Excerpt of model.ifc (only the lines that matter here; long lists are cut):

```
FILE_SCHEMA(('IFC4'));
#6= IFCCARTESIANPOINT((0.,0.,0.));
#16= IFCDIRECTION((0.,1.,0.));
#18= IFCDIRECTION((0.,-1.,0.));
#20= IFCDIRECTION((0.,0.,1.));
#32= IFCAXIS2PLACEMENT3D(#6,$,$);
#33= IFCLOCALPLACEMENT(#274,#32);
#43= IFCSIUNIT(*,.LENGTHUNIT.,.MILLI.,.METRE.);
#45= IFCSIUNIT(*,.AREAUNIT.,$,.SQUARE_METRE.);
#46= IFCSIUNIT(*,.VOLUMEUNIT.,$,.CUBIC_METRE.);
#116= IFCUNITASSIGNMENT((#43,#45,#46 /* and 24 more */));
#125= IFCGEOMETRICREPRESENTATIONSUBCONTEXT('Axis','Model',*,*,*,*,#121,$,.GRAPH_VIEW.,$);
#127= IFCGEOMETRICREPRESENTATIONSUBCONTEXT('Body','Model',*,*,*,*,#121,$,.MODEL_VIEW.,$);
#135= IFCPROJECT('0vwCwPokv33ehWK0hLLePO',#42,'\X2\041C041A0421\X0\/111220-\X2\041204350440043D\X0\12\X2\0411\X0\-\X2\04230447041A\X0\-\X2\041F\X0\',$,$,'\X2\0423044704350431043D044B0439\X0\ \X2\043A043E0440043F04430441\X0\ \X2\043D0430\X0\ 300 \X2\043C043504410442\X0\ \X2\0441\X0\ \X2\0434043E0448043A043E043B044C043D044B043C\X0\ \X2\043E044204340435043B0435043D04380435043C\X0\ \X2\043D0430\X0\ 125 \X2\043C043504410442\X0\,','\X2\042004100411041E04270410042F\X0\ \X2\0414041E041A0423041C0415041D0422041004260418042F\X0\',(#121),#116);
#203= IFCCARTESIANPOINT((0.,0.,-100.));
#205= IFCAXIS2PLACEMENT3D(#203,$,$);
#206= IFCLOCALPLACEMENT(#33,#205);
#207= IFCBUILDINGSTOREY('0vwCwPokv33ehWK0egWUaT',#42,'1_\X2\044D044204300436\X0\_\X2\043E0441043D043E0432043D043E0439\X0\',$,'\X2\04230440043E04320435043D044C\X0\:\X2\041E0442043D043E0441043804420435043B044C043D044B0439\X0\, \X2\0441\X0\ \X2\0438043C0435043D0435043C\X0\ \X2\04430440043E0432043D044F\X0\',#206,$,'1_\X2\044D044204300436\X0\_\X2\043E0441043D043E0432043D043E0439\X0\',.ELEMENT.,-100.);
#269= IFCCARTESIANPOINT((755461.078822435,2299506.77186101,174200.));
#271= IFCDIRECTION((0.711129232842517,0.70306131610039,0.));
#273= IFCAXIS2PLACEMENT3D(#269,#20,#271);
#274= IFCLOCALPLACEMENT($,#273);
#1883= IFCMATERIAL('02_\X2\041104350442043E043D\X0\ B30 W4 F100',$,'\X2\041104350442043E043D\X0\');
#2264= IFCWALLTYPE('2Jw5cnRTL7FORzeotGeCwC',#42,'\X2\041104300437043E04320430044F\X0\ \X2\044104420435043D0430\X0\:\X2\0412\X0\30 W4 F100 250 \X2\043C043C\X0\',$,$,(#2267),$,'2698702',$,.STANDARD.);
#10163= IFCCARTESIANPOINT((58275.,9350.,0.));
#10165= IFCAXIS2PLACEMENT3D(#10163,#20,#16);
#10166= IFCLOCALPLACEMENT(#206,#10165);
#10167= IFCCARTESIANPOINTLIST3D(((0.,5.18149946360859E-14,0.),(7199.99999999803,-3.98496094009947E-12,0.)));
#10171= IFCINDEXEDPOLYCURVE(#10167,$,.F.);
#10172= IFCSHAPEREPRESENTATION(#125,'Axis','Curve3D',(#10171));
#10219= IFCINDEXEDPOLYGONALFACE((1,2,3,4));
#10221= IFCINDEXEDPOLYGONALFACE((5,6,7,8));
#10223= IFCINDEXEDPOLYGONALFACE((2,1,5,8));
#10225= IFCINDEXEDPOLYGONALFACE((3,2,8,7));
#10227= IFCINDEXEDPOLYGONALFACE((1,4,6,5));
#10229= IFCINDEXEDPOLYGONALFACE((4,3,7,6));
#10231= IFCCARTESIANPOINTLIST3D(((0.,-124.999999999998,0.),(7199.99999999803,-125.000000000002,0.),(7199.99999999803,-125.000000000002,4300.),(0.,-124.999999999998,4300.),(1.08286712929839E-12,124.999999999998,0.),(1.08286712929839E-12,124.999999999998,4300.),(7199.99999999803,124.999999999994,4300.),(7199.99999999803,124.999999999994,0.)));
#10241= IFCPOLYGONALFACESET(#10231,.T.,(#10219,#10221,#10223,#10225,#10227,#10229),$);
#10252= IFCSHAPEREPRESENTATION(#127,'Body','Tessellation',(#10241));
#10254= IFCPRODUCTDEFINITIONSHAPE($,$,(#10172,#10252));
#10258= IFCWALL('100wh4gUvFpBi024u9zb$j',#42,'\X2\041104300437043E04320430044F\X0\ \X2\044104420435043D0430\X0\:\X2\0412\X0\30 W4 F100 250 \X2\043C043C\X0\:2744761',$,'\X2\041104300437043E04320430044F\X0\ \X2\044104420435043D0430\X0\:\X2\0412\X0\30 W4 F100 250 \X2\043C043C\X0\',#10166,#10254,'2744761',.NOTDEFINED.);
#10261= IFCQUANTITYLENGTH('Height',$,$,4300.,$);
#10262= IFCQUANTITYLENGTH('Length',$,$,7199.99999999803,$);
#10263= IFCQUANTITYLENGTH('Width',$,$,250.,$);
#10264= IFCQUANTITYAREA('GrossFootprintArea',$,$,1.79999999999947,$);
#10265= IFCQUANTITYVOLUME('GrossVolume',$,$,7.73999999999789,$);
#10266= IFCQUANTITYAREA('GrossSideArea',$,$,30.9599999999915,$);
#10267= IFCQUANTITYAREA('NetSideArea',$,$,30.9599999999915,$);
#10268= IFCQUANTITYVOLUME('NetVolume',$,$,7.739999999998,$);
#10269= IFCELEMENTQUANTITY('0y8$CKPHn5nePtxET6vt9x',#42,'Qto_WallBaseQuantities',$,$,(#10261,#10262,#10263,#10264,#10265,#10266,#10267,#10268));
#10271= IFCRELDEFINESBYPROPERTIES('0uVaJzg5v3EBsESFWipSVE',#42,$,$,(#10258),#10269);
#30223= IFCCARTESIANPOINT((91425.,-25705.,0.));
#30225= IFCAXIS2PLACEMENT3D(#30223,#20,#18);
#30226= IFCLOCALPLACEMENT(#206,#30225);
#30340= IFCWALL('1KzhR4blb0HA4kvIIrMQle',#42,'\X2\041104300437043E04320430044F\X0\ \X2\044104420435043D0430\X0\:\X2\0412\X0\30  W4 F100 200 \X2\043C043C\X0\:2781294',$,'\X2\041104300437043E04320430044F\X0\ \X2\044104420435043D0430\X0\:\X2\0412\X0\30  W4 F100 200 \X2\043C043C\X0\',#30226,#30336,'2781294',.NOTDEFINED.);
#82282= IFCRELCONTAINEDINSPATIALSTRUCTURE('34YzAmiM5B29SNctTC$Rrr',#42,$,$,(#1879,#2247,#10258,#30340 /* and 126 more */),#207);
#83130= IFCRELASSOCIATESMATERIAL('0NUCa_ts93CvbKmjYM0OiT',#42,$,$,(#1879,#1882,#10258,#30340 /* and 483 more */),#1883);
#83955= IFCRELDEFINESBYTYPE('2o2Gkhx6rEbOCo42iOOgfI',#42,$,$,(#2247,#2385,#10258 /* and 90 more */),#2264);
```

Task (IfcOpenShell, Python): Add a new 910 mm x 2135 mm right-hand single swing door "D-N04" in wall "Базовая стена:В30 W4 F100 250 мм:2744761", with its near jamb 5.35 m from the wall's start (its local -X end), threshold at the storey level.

```python
import numpy as np
import ifcopenshell
import ifcopenshell.api.feature
import ifcopenshell.api.geometry
import ifcopenshell.api.pset
import ifcopenshell.api.root
import ifcopenshell.api.spatial
import ifcopenshell.geom
import ifcopenshell.util.element
import ifcopenshell.util.placement
import ifcopenshell.util.representation
import ifcopenshell.util.shape
import ifcopenshell.util.unit

model = ifcopenshell.open("model.ifc")
unit_scale = ifcopenshell.util.unit.calculate_unit_scale(model)
area_scale = ifcopenshell.util.unit.calculate_unit_scale(model, "AREAUNIT")
volume_scale = ifcopenshell.util.unit.calculate_unit_scale(model, "VOLUMEUNIT")
settings = ifcopenshell.geom.settings()


def volume(element):
    """Net volume in cubic metres, openings subtracted."""
    shape = ifcopenshell.geom.create_shape(settings, element)
    return ifcopenshell.util.shape.get_volume(shape.geometry)


wall = model.by_guid("100wh4gUvFpBi024u9zb$j")
storey = ifcopenshell.util.element.get_container(wall, ifc_class="IfcBuildingStorey")
context = ifcopenshell.util.representation.get_context(model, "Model", "Body", "MODEL_VIEW")
before = volume(wall)

width, height, from_end, sill = 0.91, 2.135, 5.35, 0.0  # metres

# The wall runs along its own X axis, and the end named is its -X end.
wall_shape = ifcopenshell.geom.create_shape(settings, wall)
x, y, z = ifcopenshell.util.shape.get_vertices(wall_shape.geometry).T
start = x.min() + from_end
face, thickness = float(y.min()), float(y.max() - y.min())
wall_matrix = ifcopenshell.util.placement.get_local_placement(wall.ObjectPlacement)
level = ifcopenshell.util.placement.get_local_placement(storey.ObjectPlacement)[2, 3]


def in_wall(x, y):
    """Placement at x, y metres in the wall's axes, at sill height."""
    matrix = wall_matrix.copy()
    matrix[:, 3] = wall_matrix @ np.array([x / unit_scale, y / unit_scale, 0.0, 1.0])
    matrix[2, 3] = level + sill / unit_scale
    return matrix


# Opening: a box that overshoots both wall faces by 50 mm.
opening = ifcopenshell.api.root.create_entity(model, ifc_class="IfcOpeningElement", predefined_type="OPENING")
box = ifcopenshell.api.geometry.add_wall_representation(
    model, context=context, length=width, height=height, thickness=thickness + 0.1
)
ifcopenshell.api.geometry.assign_representation(model, product=opening, representation=box)
ifcopenshell.api.geometry.edit_object_placement(model, product=opening, matrix=in_wall(start, face - 0.05), is_si=False)
ifcopenshell.api.feature.add_feature(model, feature=opening, element=wall)

door = ifcopenshell.api.root.create_entity(model, ifc_class="IfcDoor", name="D-N04", predefined_type="DOOR")
door.OverallWidth, door.OverallHeight = width / unit_scale, height / unit_scale
door.OperationType = "SINGLE_SWING_RIGHT"
body = ifcopenshell.api.geometry.add_door_representation(
    model,
    context=context,
    overall_width=door.OverallWidth,
    overall_height=door.OverallHeight,
    operation_type="SINGLE_SWING_RIGHT",
    lining_properties={"LiningDepth": thickness / unit_scale, "ThresholdDepth": thickness / unit_scale},
)
ifcopenshell.api.geometry.assign_representation(model, product=door, representation=body)
ifcopenshell.api.spatial.assign_container(model, products=[door], relating_structure=storey)
ifcopenshell.api.feature.add_filling(model, opening=opening, element=door)

# The lining spans the wall, so the door starts at the wall face.
ifcopenshell.api.geometry.edit_object_placement(model, product=door, matrix=in_wall(start, face), is_si=False)

after = volume(wall)

# Update the wall's stored quantities.
qto = model.by_id(ifcopenshell.util.element.get_pset(wall, "Qto_WallBaseQuantities", should_inherit=False)["id"])
ifcopenshell.api.pset.edit_qto(model, qto=qto, properties={
    "NetSideArea": after / thickness / area_scale,
    "NetVolume": after / volume_scale,
})

print(f"wall volume {before:.3f} -> {after:.3f} m3")

model.write("model_updated.ifc")
```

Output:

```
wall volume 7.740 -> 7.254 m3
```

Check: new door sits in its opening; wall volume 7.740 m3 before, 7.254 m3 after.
